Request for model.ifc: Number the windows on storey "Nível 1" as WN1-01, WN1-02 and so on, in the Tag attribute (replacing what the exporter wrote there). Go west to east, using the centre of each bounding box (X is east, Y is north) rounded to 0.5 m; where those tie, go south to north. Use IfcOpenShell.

First a look at what the model holds.

```python
import ifcopenshell
import ifcopenshell.util.element
import ifcopenshell.util.placement

model = ifcopenshell.open("model.ifc")
print(model.schema)
storey = next(s for s in model.by_type("IfcBuildingStorey") if s.Name == "Nível 1")
windows = [e for e in ifcopenshell.util.element.get_decomposition(storey) if e.is_a("IfcWindow")]
for e in sorted(windows, key=lambda e: e.id()):
    origin = ifcopenshell.util.placement.get_local_placement(e.ObjectPlacement)[:3, 3]
    print(e.id(), e.Tag, e.Name, origin.round(2) + 0.0, sep=" | ")
```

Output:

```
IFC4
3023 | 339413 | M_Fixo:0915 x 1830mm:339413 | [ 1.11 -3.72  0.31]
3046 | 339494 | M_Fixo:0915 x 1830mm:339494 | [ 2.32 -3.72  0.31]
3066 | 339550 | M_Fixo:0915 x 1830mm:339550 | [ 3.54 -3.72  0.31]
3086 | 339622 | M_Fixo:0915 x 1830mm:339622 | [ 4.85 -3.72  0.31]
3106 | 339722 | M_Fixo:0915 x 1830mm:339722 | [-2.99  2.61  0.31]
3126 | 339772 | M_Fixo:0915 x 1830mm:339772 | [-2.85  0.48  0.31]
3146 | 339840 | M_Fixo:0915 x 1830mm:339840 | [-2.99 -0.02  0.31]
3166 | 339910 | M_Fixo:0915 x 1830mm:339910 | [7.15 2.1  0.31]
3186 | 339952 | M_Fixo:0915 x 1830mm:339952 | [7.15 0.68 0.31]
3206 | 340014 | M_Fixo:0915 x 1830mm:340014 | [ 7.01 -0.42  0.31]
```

```python
import ifcopenshell
import ifcopenshell.geom
import ifcopenshell.util.element
import ifcopenshell.util.shape

model = ifcopenshell.open("model.ifc")
settings = ifcopenshell.geom.settings()
settings.set("use-world-coords", True)


def centre(element):
    shape = ifcopenshell.geom.create_shape(settings, element)
    return ifcopenshell.util.shape.get_bbox_centroid(shape.geometry)


storey = next(s for s in model.by_type("IfcBuildingStorey") if s.Name == "Nível 1")
windows = [e for e in ifcopenshell.util.element.get_decomposition(storey) if e.is_a("IfcWindow")]

# Insertion points can sit at a corner or the storey origin, so sort by the geometry (in metres).
centres = {e: centre(e) for e in windows}
windows.sort(key=lambda e: (round(centres[e][0] / 0.5), centres[e][1]))

for i, e in enumerate(windows, start=1):
    number = f"WN1-{i:02d}"
    e.Tag = number
    print(e.id(), number)

model.write("model_v2.ifc")
```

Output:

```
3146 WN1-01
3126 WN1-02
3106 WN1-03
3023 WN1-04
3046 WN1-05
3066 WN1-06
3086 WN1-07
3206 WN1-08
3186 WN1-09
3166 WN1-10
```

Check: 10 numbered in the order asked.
